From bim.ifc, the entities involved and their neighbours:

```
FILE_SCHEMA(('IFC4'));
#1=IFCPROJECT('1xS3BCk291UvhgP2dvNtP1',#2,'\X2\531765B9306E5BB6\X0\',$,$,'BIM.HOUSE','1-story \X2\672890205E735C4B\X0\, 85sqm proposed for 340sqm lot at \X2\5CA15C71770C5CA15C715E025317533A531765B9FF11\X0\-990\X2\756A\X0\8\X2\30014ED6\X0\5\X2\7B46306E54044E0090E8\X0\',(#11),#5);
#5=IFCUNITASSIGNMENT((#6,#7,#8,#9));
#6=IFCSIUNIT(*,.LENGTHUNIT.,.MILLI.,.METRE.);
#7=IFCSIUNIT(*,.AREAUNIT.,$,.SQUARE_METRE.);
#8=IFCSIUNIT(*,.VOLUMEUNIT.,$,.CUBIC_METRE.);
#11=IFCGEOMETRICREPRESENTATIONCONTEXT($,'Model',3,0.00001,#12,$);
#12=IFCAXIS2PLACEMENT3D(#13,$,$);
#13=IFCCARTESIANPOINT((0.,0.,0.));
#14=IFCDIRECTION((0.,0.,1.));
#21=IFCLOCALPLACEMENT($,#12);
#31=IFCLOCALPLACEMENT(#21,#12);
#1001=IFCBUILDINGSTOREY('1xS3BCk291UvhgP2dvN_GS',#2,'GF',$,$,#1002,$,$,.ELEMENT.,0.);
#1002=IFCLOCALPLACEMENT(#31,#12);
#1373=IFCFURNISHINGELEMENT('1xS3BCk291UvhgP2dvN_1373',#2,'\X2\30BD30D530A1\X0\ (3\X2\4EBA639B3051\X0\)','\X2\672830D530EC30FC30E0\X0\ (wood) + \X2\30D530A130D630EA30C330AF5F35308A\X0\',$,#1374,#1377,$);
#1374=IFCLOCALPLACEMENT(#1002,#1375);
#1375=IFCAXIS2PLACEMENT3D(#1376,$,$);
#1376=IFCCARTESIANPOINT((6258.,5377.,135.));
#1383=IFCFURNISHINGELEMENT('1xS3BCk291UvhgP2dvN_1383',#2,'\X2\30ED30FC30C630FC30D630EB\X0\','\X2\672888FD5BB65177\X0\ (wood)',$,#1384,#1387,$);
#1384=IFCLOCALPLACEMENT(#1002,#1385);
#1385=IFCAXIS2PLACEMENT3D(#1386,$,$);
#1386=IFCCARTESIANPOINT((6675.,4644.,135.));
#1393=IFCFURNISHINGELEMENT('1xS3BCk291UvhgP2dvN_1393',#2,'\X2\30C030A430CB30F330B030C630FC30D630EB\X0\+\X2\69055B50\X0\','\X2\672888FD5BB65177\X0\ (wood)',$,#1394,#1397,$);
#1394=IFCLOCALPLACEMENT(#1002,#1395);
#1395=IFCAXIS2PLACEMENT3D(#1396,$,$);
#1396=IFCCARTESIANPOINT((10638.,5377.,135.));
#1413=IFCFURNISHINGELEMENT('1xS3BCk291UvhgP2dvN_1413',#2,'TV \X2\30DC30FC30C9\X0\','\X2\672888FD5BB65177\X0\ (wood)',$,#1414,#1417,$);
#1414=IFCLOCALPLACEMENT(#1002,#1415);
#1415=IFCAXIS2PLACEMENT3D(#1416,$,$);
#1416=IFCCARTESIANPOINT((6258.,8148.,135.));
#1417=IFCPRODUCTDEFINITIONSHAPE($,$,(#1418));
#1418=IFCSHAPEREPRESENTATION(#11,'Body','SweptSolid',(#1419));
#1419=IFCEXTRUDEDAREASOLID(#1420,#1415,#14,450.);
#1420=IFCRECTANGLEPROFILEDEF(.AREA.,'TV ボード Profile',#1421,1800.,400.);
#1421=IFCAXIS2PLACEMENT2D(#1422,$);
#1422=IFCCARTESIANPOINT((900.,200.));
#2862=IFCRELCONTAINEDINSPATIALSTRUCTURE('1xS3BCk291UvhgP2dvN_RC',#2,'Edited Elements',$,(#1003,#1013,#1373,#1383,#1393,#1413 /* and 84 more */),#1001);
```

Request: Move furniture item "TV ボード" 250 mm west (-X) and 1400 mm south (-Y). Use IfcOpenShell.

```python
import ifcopenshell
import ifcopenshell.api.geometry
import ifcopenshell.util.placement

model = ifcopenshell.open("bim.ifc")

item = model.by_guid("1xS3BCk291UvhgP2dvN_1413")
matrix = ifcopenshell.util.placement.get_local_placement(item.ObjectPlacement)
matrix[0, 3] -= 250.0
matrix[1, 3] -= 1400.0
ifcopenshell.api.geometry.edit_object_placement(model, product=item, matrix=matrix, is_si=False)

print(ifcopenshell.util.placement.get_local_placement(item.ObjectPlacement).round(3) + 0.0)

model.write("bim_v2.ifc")
```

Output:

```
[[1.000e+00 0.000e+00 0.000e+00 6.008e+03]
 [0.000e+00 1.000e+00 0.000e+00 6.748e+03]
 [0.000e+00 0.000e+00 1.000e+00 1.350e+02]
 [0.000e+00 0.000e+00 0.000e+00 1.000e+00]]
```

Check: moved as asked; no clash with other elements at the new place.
